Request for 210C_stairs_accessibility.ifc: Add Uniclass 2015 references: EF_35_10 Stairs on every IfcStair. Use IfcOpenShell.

First a look at what the model holds.

```python
import ifcopenshell

model = ifcopenshell.open("210C_stairs_accessibility.ifc")
print(model.schema)
print("classifications:", [c.Name for c in model.by_type("IfcClassification")])
for ifc_class in ("IfcDoor", "IfcRoof", "IfcStair", "IfcWall", "IfcWindow"):
    print(ifc_class, len(model.by_type(ifc_class)))
```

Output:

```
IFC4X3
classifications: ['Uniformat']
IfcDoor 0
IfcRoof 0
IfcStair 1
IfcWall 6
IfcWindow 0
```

```python
import ifcopenshell
import ifcopenshell.api.classification

model = ifcopenshell.open("210C_stairs_accessibility.ifc")

system = ifcopenshell.api.classification.add_classification(model, classification="Uniclass 2015")

codes = {
    "IfcStair": ("EF_35_10", "Stairs"),
}
for ifc_class, (code, name) in codes.items():
    products = model.by_type(ifc_class)
    ifcopenshell.api.classification.add_reference(
        model, products=products, classification=system, identification=code, name=name
    )
    print(code, len(products))

model.write("210C_stairs_accessibility-out.ifc")
```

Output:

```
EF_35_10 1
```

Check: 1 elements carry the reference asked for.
